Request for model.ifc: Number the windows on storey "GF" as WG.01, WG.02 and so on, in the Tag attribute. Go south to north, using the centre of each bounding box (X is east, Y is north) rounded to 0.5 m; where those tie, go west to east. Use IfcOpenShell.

First a look at what the model holds.

```python
import ifcopenshell
import ifcopenshell.util.element
import ifcopenshell.util.placement

model = ifcopenshell.open("model.ifc")
print(model.schema)
storey = next(s for s in model.by_type("IfcBuildingStorey") if s.Name == "GF")
windows = [e for e in ifcopenshell.util.element.get_decomposition(storey) if e.is_a("IfcWindow")]
for e in sorted(windows, key=lambda e: e.id()):
    origin = ifcopenshell.util.placement.get_local_placement(e.ObjectPlacement)[:3, 3]
    print(e.id(), e.Tag, e.Name, origin.round(2) + 0.0, sep=" | ")
```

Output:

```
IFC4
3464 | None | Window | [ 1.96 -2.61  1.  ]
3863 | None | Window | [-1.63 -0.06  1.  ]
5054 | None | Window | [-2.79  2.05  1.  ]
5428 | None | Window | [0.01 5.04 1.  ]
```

```python
import ifcopenshell
import ifcopenshell.geom
import ifcopenshell.util.element
import ifcopenshell.util.shape

model = ifcopenshell.open("model.ifc")
settings = ifcopenshell.geom.settings()
settings.set("use-world-coords", True)


def centre(element):
    shape = ifcopenshell.geom.create_shape(settings, element)
    return ifcopenshell.util.shape.get_bbox_centroid(shape.geometry)


storey = next(s for s in model.by_type("IfcBuildingStorey") if s.Name == "GF")
windows = [e for e in ifcopenshell.util.element.get_decomposition(storey) if e.is_a("IfcWindow")]

# Insertion points can sit at a corner or the storey origin, so sort by the geometry (in metres).
centres = {e: centre(e) for e in windows}
windows.sort(key=lambda e: (round(centres[e][1] / 0.5), centres[e][0]))

for i, e in enumerate(windows, start=1):
    number = f"WG.{i:02d}"
    e.Tag = number
    print(e.id(), number)

model.write("model-out.ifc")
```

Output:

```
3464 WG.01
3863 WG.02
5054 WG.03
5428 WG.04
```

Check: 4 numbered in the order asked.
